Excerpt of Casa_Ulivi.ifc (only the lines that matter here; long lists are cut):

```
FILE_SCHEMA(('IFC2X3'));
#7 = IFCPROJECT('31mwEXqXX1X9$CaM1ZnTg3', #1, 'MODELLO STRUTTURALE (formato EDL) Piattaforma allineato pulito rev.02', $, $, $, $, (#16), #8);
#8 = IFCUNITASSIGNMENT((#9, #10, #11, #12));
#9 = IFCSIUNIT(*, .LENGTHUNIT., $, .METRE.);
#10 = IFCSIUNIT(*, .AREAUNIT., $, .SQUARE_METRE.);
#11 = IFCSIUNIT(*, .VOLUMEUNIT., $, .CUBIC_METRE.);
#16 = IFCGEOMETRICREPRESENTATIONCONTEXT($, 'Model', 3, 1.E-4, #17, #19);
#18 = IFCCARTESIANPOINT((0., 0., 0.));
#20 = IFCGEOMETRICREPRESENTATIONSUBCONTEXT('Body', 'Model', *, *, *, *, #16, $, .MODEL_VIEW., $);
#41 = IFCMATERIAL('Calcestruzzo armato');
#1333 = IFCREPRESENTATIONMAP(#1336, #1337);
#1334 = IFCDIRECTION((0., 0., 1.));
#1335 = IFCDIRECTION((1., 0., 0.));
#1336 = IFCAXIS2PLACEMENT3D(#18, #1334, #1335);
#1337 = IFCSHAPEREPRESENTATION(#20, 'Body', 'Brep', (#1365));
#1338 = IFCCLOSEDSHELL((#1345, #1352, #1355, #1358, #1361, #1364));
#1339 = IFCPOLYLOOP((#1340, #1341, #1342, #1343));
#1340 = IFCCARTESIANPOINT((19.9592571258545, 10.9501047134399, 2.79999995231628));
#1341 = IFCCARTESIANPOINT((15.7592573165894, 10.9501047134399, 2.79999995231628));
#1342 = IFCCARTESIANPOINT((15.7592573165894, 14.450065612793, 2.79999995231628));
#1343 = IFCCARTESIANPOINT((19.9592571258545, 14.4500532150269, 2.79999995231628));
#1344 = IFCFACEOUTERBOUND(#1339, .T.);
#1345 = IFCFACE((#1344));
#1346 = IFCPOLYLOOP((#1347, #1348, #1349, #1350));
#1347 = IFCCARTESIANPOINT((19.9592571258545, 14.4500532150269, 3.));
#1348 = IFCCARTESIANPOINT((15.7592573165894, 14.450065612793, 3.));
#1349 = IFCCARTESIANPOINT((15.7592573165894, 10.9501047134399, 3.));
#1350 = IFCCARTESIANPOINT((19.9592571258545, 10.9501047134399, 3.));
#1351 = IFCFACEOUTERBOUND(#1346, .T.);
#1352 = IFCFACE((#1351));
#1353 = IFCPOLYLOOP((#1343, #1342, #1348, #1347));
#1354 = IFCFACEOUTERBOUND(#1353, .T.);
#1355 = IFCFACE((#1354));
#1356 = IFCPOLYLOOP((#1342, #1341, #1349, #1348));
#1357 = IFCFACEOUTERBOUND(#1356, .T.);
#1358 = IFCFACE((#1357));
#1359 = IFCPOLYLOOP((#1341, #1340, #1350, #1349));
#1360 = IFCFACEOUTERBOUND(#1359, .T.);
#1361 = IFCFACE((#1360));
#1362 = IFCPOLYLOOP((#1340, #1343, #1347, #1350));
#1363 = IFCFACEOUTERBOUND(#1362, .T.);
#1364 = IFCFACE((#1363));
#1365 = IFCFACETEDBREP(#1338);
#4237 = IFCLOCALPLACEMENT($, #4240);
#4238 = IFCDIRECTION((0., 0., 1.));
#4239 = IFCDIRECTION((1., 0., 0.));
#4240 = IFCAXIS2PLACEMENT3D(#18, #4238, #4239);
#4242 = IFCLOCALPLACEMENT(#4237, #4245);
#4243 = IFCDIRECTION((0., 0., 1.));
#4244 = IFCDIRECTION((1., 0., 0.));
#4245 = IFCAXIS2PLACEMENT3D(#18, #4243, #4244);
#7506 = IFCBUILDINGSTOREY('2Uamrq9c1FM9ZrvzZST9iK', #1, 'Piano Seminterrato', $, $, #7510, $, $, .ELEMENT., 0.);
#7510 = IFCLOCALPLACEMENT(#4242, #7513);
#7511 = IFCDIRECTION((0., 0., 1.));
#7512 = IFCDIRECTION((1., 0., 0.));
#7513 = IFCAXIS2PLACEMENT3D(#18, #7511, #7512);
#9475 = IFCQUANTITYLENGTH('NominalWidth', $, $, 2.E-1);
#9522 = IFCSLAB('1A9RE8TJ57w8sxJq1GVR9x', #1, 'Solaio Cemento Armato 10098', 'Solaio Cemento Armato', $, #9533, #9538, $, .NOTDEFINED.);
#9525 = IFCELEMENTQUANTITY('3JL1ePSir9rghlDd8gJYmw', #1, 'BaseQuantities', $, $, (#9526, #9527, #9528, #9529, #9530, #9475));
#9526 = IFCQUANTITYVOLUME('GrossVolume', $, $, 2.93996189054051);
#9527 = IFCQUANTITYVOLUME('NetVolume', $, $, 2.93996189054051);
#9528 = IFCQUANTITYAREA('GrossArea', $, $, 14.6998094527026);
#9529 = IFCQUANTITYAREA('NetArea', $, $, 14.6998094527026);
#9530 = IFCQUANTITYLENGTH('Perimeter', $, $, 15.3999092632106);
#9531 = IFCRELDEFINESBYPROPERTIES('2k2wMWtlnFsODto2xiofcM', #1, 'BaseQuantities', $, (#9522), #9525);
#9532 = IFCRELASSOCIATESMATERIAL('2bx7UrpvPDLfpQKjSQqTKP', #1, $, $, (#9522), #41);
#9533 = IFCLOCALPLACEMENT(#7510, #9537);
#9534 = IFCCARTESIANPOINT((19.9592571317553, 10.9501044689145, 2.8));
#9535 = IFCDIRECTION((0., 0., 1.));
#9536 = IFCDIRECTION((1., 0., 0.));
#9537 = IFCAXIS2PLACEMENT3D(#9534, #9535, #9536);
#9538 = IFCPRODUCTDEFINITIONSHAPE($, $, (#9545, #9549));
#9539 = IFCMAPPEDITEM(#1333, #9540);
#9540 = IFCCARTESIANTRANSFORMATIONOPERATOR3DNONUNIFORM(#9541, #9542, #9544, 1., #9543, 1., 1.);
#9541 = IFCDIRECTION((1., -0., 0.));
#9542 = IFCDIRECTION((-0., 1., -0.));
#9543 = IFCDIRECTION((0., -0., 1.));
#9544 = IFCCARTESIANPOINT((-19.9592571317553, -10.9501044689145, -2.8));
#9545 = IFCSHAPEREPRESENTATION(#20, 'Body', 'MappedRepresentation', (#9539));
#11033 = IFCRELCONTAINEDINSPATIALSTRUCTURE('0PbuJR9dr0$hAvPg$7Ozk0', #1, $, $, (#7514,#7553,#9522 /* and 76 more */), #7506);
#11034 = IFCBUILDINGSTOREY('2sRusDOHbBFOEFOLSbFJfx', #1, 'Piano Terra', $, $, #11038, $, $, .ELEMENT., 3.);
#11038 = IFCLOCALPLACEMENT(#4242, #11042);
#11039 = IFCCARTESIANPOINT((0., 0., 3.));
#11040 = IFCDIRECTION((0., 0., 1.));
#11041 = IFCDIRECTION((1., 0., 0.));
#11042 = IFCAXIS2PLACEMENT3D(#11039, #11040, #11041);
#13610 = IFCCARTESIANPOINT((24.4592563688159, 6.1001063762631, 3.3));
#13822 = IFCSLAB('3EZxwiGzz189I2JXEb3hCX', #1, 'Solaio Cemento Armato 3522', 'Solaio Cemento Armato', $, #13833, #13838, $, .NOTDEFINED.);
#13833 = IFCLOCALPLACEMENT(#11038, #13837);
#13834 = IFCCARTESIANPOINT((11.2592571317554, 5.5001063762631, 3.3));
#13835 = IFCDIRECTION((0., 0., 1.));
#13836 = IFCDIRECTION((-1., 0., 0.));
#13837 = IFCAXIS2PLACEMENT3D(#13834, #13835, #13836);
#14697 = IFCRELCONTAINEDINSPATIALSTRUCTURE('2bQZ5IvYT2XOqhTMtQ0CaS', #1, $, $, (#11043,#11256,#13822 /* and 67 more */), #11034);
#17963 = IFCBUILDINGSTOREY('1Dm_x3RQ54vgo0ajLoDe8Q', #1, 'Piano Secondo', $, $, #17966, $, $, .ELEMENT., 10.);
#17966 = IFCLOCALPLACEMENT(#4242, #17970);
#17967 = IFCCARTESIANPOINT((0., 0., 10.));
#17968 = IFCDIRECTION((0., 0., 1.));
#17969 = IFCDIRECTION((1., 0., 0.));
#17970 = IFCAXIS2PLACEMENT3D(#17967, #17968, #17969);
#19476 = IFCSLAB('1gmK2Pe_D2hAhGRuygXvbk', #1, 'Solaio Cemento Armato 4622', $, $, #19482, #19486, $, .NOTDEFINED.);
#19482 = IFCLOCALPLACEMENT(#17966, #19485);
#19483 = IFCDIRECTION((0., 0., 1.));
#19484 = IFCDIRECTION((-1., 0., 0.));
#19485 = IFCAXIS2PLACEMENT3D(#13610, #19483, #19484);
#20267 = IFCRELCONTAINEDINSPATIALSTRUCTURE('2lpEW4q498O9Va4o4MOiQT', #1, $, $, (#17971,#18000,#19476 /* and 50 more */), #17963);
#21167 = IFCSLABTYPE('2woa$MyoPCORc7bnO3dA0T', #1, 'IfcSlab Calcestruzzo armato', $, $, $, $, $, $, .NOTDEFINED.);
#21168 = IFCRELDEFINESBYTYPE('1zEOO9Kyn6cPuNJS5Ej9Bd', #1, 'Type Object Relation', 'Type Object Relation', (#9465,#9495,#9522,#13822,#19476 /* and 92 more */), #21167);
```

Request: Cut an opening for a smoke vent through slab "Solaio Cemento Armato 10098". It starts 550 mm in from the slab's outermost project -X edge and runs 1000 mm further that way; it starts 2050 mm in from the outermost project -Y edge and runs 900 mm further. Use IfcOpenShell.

```python
import numpy as np
import ifcopenshell
import ifcopenshell.api.feature
import ifcopenshell.api.geometry
import ifcopenshell.api.pset
import ifcopenshell.api.root
import ifcopenshell.geom
import ifcopenshell.util.element
import ifcopenshell.util.placement
import ifcopenshell.util.representation
import ifcopenshell.util.shape
import ifcopenshell.util.unit

model = ifcopenshell.open("Casa_Ulivi.ifc")
unit_scale = ifcopenshell.util.unit.calculate_unit_scale(model)
area_scale = ifcopenshell.util.unit.calculate_unit_scale(model, "AREAUNIT")
volume_scale = ifcopenshell.util.unit.calculate_unit_scale(model, "VOLUMEUNIT")
settings = ifcopenshell.geom.settings()


def volume(element):
    """Net volume in cubic metres, openings subtracted."""
    shape = ifcopenshell.geom.create_shape(settings, element)
    return ifcopenshell.util.shape.get_volume(shape.geometry)


slab = model.by_guid("1A9RE8TJ57w8sxJq1GVR9x")
before = volume(slab)

# Extent in the slab's own axes, in metres. The edges named are its -X and -Y sides.
slab_shape = ifcopenshell.geom.create_shape(settings, slab)
vertices = ifcopenshell.util.shape.get_vertices(slab_shape.geometry)
x_min, y_min, bottom = vertices.min(axis=0)
top = vertices[:, 2].max()

opening = ifcopenshell.api.root.create_entity(model, ifc_class="IfcOpeningElement", name="Smoke vent opening")
context = ifcopenshell.util.representation.get_context(model, "Model", "Body", "MODEL_VIEW")
width, depth = 1, 0.9
outline = [(0.0, 0.0), (width, 0.0), (width, depth), (0.0, depth), (0.0, 0.0)]
# Overshoot both faces by 50 mm so the cut is clean.
shape = ifcopenshell.api.geometry.add_slab_representation(
    model, context=context, depth=top - bottom + 0.1, polyline=outline
)
ifcopenshell.api.geometry.assign_representation(model, product=opening, representation=shape)

matrix = ifcopenshell.util.placement.get_local_placement(slab.ObjectPlacement)
matrix[:, 3] = matrix @ np.append(np.array([x_min + 0.55, y_min + 2.05, bottom - 0.05]) / unit_scale, 1.0)
ifcopenshell.api.geometry.edit_object_placement(model, product=opening, matrix=matrix, is_si=False)
ifcopenshell.api.feature.add_feature(model, feature=opening, element=slab)

after = volume(slab)

# Update the slab's stored quantities.
qto = model.by_id(ifcopenshell.util.element.get_pset(slab, "BaseQuantities", should_inherit=False)["id"])
ifcopenshell.api.pset.edit_qto(model, qto=qto, properties={
    "NetVolume": after / volume_scale,
    "NetArea": after / (top - bottom) / area_scale,
})

print(f"slab volume {before:.3f} -> {after:.3f} m3")

model.write("Casa_Ulivi_updated.ifc")
```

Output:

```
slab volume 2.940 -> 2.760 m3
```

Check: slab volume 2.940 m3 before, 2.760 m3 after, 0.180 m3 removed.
